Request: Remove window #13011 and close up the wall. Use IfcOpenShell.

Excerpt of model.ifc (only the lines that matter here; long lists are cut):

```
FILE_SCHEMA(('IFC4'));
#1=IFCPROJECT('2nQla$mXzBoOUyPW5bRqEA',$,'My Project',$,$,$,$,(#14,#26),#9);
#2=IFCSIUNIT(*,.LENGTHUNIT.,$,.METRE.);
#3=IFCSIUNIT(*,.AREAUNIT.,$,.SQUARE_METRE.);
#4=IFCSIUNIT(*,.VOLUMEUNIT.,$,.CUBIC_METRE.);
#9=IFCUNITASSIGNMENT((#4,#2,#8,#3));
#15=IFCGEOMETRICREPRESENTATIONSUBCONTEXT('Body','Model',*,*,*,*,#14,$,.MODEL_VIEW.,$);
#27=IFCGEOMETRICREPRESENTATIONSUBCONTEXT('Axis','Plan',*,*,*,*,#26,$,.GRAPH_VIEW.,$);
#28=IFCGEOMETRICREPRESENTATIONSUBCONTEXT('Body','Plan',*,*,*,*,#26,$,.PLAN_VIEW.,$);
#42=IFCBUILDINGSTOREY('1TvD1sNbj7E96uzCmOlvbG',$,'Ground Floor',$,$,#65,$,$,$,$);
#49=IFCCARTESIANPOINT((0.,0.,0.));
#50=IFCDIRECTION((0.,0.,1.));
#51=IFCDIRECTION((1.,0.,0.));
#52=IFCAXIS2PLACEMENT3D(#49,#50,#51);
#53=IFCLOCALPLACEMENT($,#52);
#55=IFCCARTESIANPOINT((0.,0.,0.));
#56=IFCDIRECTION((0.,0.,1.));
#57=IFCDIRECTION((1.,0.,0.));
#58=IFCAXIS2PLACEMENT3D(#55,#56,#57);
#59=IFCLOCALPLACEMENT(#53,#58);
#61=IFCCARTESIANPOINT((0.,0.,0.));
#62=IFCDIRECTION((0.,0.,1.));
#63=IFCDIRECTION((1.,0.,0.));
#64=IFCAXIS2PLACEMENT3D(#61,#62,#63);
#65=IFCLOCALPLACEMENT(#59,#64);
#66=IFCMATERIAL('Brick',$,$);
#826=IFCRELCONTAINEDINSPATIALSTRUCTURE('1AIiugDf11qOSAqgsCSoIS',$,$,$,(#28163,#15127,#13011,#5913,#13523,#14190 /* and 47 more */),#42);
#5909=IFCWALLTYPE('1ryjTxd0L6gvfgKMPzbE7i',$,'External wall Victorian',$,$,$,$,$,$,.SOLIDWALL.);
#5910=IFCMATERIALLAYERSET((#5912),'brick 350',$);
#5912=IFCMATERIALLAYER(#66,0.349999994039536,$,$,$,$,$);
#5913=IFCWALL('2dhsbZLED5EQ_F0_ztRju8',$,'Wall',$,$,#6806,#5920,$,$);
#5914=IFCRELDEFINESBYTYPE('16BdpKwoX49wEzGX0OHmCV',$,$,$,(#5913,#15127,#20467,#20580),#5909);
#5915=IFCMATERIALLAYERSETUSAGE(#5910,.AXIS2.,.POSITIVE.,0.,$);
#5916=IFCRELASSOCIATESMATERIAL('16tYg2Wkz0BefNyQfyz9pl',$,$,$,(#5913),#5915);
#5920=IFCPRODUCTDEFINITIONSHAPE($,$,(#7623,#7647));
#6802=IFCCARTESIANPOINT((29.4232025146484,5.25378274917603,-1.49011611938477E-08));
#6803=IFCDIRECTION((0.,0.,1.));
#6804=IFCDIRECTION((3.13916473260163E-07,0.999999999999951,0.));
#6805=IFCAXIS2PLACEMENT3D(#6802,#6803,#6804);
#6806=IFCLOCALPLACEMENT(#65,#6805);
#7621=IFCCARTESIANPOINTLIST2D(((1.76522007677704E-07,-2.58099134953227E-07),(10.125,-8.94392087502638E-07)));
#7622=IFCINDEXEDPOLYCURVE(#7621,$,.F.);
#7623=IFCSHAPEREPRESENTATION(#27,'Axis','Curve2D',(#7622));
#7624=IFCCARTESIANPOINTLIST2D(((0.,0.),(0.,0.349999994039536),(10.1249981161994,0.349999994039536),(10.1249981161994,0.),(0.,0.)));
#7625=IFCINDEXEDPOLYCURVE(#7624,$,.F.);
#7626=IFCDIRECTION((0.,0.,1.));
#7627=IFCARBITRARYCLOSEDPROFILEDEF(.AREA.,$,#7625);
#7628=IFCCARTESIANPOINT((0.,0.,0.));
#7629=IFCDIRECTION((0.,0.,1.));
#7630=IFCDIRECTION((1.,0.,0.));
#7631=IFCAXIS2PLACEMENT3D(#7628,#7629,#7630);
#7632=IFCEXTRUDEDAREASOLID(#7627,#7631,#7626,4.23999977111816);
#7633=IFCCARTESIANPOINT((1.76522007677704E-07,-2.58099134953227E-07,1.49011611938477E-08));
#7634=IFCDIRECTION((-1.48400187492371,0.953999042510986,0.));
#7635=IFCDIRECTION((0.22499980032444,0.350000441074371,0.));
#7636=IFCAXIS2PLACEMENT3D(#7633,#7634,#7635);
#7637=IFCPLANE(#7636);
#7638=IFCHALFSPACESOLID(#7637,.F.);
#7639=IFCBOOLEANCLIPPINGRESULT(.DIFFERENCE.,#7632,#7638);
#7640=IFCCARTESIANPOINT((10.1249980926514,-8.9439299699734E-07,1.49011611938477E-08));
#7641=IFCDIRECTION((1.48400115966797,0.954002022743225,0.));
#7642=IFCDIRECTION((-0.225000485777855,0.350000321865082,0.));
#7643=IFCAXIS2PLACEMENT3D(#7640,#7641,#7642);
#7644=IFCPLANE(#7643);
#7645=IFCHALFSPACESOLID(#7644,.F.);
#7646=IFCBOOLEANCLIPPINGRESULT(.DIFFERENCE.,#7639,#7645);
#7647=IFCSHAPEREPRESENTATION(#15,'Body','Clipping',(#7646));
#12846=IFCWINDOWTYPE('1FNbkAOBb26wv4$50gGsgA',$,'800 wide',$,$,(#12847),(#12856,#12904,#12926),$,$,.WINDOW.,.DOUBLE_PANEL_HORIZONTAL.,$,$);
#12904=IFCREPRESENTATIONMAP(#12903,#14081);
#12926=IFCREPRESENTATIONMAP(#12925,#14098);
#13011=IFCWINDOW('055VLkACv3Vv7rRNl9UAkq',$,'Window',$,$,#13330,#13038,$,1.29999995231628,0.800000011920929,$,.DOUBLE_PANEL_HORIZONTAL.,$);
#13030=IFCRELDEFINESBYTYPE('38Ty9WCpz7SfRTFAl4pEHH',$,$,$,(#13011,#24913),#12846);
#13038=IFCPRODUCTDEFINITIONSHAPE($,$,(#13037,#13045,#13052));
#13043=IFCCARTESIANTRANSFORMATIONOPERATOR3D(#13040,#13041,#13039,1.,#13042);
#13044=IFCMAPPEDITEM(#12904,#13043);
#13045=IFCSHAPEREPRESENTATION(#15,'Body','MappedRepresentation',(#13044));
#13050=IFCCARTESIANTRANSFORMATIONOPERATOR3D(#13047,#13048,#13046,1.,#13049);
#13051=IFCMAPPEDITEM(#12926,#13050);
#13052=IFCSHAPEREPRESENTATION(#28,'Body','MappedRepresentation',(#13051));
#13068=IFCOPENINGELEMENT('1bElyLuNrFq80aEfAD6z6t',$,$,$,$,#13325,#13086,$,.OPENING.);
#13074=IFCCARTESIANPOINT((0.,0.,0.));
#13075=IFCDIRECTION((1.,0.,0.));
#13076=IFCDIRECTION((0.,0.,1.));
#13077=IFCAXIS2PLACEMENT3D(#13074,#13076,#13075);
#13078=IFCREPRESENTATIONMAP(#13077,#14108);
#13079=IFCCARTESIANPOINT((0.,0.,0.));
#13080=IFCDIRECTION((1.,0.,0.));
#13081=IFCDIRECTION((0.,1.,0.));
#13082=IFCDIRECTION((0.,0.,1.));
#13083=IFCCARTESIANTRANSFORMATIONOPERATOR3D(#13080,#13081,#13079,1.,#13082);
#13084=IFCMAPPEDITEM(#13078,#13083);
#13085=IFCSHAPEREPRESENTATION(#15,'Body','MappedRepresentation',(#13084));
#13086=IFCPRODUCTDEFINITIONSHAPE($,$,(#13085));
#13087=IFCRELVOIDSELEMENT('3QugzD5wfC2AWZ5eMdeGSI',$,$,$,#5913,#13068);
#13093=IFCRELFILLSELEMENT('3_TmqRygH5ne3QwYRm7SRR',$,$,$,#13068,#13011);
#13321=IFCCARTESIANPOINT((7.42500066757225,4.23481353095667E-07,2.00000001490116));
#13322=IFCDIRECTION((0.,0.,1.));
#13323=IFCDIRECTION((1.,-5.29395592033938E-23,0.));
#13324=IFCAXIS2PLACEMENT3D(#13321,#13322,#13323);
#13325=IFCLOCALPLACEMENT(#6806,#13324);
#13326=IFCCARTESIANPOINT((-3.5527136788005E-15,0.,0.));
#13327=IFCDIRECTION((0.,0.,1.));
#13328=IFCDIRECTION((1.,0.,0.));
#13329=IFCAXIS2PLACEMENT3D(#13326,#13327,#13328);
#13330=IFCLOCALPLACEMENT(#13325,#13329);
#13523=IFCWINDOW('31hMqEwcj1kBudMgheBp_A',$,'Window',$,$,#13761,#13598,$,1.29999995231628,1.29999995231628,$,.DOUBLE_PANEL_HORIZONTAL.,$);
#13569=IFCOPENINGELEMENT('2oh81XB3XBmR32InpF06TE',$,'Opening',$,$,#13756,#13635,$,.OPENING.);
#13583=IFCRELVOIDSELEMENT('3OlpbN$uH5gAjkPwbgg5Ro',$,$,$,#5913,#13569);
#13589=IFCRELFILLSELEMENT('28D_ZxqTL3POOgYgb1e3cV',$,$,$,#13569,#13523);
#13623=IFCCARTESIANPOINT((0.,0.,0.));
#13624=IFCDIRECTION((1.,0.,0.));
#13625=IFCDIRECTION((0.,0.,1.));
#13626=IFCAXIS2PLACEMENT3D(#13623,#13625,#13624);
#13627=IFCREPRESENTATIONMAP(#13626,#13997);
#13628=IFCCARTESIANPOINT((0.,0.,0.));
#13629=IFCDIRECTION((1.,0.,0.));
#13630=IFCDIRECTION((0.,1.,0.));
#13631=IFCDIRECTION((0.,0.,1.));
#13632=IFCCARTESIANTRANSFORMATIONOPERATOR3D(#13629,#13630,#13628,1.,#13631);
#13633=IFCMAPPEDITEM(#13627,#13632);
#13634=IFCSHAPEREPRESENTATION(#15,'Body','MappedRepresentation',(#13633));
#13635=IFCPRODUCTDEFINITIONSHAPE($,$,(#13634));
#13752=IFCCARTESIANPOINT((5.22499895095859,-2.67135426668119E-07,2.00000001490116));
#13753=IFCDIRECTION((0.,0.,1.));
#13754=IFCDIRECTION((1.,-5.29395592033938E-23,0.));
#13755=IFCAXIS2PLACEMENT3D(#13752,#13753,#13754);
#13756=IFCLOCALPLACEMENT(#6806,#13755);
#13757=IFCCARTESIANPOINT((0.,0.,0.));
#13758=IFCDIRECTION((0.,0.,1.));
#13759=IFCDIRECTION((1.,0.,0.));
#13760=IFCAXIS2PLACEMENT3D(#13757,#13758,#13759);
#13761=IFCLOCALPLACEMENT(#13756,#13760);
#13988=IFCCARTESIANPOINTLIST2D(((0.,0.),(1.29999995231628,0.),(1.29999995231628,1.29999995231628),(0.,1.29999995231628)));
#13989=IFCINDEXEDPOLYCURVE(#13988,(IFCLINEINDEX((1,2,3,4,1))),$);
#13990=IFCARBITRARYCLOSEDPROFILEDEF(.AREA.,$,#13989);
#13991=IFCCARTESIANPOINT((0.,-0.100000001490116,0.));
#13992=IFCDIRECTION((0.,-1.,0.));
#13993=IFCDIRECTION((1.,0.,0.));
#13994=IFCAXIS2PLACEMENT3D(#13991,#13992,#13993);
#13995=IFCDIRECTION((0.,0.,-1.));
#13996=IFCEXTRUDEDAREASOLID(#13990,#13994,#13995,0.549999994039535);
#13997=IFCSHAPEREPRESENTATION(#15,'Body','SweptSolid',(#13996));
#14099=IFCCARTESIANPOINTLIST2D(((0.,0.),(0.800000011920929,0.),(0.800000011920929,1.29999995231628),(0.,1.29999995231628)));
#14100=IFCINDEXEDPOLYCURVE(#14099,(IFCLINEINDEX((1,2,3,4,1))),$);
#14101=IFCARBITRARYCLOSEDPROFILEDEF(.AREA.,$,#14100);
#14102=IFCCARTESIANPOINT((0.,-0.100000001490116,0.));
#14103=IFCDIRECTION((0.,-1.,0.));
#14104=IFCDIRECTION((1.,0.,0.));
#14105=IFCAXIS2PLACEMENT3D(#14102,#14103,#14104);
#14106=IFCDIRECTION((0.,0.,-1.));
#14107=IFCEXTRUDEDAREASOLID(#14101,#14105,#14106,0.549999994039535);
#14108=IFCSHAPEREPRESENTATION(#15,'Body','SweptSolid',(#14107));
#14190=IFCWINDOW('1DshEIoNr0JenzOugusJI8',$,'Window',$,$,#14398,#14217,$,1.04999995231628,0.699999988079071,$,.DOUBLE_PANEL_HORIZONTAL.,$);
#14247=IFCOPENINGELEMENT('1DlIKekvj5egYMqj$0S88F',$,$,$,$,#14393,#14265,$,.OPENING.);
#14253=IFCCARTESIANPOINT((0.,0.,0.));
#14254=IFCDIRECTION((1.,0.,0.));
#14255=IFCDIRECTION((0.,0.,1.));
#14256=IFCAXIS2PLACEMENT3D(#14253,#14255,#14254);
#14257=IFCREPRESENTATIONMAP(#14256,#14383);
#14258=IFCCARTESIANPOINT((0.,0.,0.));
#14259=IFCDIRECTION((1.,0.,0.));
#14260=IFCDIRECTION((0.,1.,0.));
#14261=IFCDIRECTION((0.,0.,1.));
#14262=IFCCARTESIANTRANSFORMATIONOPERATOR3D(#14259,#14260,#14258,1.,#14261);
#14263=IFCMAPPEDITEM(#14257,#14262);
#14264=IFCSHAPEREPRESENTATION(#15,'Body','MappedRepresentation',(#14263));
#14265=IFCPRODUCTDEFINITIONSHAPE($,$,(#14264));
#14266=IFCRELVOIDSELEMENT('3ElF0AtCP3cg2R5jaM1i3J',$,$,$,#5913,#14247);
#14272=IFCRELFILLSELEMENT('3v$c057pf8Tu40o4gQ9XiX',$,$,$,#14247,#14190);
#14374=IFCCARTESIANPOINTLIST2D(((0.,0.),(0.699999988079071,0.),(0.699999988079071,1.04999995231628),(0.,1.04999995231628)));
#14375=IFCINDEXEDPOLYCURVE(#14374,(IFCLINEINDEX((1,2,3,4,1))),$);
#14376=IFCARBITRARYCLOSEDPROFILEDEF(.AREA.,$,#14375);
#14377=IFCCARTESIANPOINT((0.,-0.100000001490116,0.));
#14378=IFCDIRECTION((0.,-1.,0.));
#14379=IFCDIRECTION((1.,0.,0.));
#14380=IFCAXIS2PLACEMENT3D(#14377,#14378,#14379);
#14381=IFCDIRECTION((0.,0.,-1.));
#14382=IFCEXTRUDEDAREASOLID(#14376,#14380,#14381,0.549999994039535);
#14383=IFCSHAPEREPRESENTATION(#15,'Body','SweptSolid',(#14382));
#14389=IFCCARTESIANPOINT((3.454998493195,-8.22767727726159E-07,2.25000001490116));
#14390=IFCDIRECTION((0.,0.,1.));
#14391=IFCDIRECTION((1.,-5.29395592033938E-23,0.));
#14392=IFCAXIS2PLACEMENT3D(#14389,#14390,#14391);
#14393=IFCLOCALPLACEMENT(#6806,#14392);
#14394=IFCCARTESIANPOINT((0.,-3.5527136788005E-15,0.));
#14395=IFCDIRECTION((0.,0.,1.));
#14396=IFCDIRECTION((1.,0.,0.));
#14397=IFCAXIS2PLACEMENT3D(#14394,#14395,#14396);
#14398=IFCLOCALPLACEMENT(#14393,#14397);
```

```python
import ifcopenshell
import ifcopenshell.api.feature
import ifcopenshell.api.root
import ifcopenshell.geom
import ifcopenshell.util.shape

model = ifcopenshell.open("model.ifc")
settings = ifcopenshell.geom.settings()


def volume(element):
    """Net volume in cubic metres, openings subtracted."""
    shape = ifcopenshell.geom.create_shape(settings, element)
    return ifcopenshell.util.shape.get_volume(shape.geometry)


window = model.by_id(13011)
opening = window.FillsVoids[0].RelatingOpeningElement
wall = opening.VoidsElements[0].RelatingBuildingElement
before = volume(wall)

ifcopenshell.api.root.remove_product(model, product=window)
ifcopenshell.api.feature.remove_feature(model, feature=opening)

after = volume(wall)

print(f"wall volume {before:.3f} -> {after:.3f} m3")

model.write("model-out.ifc")
```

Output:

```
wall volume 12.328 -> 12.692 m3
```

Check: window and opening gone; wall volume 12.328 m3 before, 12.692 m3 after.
